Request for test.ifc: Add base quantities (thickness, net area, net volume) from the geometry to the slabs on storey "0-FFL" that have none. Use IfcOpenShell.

First a look at what the model holds.

```python
import ifcopenshell
import ifcopenshell.util.element
import ifcopenshell.util.unit

model = ifcopenshell.open("test.ifc")
print(model.schema)
for unit_type in ("LENGTHUNIT", "AREAUNIT", "VOLUMEUNIT"):
    print(unit_type, ifcopenshell.util.unit.calculate_unit_scale(model, unit_type))
storey = next(s for s in model.by_type("IfcBuildingStorey") if s.Name == "0-FFL")
slabs = [e for e in ifcopenshell.util.element.get_decomposition(storey) if e.is_a("IfcSlab")]
for e in sorted(slabs, key=lambda e: e.id()):
    print(e.id(), e.is_a(), e.Name, list(ifcopenshell.util.element.get_psets(e, qtos_only=True)), sep=" | ")
```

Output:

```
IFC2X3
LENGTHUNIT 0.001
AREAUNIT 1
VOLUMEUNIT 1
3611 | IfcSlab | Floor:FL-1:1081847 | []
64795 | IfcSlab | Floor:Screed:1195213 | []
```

```python
import ifcopenshell
import ifcopenshell.api.pset
import ifcopenshell.geom
import ifcopenshell.util.element
import ifcopenshell.util.shape
import ifcopenshell.util.unit

model = ifcopenshell.open("test.ifc")
unit_scale = ifcopenshell.util.unit.calculate_unit_scale(model)
area_scale = ifcopenshell.util.unit.calculate_unit_scale(model, "AREAUNIT")
volume_scale = ifcopenshell.util.unit.calculate_unit_scale(model, "VOLUMEUNIT")
settings = ifcopenshell.geom.settings()

storey = next(s for s in model.by_type("IfcBuildingStorey") if s.Name == "0-FFL")
slabs = [e for e in ifcopenshell.util.element.get_decomposition(storey) if e.is_a("IfcSlab")]

for e in sorted(slabs, key=lambda e: e.id()):
    if ifcopenshell.util.element.get_psets(e, qtos_only=True, should_inherit=False):
        continue
    # Geometry comes back in metres, in the element's own axes.
    shape = ifcopenshell.geom.create_shape(settings, e)
    values = {
        "Width": ifcopenshell.util.shape.get_z(shape.geometry) / unit_scale,
        "NetArea": ifcopenshell.util.shape.get_footprint_area(shape.geometry) / area_scale,
        "NetVolume": ifcopenshell.util.shape.get_volume(shape.geometry) / volume_scale,
    }
    qto = ifcopenshell.api.pset.add_qto(model, product=e, name="BaseQuantities")
    ifcopenshell.api.pset.edit_qto(model, qto=qto, properties=values)
    print(e.id(), {k: round(v, 3) for k, v in values.items()})

model.write("test_rev.ifc")
```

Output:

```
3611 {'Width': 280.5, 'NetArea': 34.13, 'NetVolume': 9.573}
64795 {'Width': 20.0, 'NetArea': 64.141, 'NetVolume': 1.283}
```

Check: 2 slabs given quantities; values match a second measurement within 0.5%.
